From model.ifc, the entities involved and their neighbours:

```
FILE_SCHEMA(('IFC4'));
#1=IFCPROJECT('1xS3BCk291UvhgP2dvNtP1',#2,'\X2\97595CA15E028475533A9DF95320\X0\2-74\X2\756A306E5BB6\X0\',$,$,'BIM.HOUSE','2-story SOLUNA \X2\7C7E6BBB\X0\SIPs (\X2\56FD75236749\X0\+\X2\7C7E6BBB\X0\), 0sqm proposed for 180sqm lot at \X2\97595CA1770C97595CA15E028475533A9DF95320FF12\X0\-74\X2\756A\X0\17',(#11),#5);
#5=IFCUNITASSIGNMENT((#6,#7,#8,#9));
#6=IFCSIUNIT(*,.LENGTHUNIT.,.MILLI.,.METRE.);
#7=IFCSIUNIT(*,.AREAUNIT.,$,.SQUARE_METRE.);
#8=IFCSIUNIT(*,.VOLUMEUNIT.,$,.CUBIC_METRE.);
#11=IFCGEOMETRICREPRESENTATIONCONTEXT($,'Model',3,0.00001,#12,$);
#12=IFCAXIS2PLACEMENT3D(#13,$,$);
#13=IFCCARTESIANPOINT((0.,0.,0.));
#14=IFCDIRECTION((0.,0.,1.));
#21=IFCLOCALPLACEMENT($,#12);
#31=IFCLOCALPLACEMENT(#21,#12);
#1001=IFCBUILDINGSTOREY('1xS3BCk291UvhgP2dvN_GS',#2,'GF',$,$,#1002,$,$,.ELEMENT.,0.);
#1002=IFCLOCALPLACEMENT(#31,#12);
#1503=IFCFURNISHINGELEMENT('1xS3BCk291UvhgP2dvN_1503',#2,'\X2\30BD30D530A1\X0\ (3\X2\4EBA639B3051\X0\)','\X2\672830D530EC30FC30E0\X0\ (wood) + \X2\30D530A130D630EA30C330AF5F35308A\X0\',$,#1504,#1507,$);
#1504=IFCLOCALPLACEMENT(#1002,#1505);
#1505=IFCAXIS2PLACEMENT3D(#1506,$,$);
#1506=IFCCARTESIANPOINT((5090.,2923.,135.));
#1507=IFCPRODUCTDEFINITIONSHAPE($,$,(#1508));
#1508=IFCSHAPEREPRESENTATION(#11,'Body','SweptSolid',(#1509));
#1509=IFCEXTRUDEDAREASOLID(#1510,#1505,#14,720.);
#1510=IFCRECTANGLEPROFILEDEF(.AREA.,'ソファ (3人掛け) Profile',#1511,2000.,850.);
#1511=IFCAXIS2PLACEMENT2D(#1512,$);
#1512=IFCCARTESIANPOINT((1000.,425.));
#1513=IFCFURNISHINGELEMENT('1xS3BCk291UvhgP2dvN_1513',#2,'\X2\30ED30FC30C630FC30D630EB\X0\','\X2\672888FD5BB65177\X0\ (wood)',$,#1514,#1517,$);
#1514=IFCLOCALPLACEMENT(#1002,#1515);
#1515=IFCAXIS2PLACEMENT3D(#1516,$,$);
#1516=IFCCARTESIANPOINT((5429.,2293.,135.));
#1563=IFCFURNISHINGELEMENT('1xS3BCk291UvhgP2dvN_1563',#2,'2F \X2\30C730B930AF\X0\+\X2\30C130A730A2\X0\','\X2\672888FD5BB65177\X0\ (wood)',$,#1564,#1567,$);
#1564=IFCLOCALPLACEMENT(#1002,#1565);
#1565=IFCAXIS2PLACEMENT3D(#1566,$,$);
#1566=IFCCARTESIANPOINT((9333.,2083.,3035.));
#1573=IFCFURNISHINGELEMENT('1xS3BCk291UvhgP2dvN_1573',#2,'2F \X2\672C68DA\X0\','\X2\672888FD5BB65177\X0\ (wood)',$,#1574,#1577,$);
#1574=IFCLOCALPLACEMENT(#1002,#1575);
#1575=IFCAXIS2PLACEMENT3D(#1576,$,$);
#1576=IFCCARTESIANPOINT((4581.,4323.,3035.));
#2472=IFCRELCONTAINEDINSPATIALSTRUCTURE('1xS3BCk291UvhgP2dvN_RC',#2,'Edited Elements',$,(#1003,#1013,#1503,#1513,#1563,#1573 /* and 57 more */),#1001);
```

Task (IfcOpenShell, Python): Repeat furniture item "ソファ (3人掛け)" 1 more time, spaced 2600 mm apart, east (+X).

```python
import numpy as np
import ifcopenshell
import ifcopenshell.api.geometry
import ifcopenshell.api.root
import ifcopenshell.util.element
import ifcopenshell.util.placement
import ifcopenshell.util.unit

model = ifcopenshell.open("model.ifc")
unit_scale = ifcopenshell.util.unit.calculate_unit_scale(model)


def reuse_history(source, copy):
    """copy_class also copies each property set's owner history, people and application; keep the originals."""
    for rel in copy.IsDefinedBy:
        if rel.is_a("IfcRelDefinesByProperties") and (history := rel.RelatingPropertyDefinition.OwnerHistory):
            rel.RelatingPropertyDefinition.OwnerHistory = source.OwnerHistory
            ifcopenshell.util.element.remove_deep2(model, history)


source = model.by_id(1503)
base = ifcopenshell.util.placement.get_local_placement(source.ObjectPlacement)
step = np.array([1.0, 0.0, 0.0]) * 2.6 / unit_scale

for i in range(1, 2):
    copy = ifcopenshell.api.root.copy_class(model, product=source)
    copy.Representation = ifcopenshell.util.element.copy_deep(
        model, source.Representation, exclude=["IfcGeometricRepresentationContext", "IfcRepresentationMap"]
    )
    reuse_history(source, copy)
    matrix = base.copy()
    matrix[:3, 3] += i * step
    print("added at", matrix[:3, 3].round(3) + 0.0)
    ifcopenshell.api.geometry.edit_object_placement(model, product=copy, matrix=matrix, is_si=False)

model.write("model-out.ifc")
```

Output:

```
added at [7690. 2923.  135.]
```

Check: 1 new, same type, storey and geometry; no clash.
